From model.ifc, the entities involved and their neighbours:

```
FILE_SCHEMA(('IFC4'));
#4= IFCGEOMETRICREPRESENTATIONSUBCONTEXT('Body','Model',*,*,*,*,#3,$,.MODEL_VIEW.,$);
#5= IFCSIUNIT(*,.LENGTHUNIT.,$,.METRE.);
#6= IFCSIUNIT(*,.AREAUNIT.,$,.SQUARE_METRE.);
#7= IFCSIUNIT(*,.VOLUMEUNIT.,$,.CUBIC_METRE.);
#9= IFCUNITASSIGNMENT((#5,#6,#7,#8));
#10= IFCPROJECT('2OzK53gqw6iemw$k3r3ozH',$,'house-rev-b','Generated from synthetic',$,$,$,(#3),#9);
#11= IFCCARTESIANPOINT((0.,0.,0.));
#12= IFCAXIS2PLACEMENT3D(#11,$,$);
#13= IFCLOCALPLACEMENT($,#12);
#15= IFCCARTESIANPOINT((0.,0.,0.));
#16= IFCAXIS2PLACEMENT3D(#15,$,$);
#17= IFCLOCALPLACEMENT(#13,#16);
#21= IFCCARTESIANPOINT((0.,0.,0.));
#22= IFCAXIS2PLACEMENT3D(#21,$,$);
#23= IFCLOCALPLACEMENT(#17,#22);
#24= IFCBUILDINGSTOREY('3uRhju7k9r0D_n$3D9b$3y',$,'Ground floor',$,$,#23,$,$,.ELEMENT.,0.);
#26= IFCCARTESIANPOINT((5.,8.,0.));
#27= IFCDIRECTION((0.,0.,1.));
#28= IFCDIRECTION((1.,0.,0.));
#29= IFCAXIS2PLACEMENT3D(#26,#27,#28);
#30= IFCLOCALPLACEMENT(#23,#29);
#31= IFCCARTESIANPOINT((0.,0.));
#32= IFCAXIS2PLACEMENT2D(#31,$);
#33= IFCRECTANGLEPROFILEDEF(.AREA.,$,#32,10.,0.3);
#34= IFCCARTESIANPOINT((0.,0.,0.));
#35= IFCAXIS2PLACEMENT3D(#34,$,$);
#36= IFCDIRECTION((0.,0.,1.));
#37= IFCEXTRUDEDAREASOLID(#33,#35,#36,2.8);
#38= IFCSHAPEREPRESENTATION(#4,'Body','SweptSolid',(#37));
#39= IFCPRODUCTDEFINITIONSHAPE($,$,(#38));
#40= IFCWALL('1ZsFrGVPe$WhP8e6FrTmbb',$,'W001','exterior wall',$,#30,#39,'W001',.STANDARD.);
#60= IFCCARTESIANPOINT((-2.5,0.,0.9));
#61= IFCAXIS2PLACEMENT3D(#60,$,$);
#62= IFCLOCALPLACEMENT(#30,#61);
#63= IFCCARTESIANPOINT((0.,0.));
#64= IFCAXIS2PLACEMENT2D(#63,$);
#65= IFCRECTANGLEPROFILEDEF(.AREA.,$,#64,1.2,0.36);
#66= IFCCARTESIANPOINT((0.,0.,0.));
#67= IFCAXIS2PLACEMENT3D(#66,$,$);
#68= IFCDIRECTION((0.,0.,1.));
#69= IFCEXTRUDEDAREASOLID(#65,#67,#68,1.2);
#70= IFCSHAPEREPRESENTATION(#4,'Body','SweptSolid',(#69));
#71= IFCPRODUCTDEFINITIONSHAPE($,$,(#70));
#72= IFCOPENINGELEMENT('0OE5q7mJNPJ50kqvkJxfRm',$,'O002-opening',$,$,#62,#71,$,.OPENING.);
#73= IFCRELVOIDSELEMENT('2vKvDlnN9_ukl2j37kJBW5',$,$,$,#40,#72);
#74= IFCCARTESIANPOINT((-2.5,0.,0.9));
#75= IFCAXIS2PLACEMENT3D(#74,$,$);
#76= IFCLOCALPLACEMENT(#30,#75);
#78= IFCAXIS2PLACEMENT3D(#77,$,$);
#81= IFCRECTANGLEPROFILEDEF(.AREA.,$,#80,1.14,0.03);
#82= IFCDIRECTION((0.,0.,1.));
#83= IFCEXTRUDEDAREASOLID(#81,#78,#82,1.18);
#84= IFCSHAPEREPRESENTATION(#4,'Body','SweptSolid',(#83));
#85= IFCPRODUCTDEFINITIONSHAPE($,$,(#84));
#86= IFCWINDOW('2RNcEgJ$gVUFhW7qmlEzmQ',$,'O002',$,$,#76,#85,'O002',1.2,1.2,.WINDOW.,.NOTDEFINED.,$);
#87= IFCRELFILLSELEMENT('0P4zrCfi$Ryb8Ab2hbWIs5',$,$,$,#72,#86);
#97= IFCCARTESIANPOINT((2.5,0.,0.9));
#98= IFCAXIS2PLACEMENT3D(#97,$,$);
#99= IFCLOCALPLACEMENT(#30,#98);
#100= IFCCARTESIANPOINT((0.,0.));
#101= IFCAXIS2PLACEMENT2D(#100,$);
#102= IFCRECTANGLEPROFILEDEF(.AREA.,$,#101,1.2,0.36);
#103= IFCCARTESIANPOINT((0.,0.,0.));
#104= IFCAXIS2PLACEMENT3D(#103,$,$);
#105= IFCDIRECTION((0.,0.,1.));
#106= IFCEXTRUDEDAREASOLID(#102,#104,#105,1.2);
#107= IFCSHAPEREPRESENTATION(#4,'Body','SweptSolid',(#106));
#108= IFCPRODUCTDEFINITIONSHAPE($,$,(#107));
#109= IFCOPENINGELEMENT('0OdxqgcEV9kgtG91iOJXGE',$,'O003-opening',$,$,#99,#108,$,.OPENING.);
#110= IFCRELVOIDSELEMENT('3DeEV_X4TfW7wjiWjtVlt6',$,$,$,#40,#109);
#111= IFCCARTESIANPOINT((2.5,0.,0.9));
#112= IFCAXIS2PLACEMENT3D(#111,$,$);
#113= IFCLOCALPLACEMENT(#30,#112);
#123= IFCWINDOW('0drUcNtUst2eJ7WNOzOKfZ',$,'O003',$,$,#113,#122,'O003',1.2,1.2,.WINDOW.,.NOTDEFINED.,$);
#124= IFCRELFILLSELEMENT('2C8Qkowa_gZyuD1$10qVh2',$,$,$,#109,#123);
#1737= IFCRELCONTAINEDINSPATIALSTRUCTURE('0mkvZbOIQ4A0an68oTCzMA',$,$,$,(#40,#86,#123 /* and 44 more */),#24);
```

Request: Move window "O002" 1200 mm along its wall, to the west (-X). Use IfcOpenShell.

```python
import ifcopenshell
import ifcopenshell.api.geometry
import ifcopenshell.util.placement
import ifcopenshell.util.unit

model = ifcopenshell.open("model.ifc")
unit_scale = ifcopenshell.util.unit.calculate_unit_scale(model)

window = model.by_guid("2RNcEgJ$gVUFhW7qmlEzmQ")
opening = window.FillsVoids[0].RelatingOpeningElement
wall = opening.VoidsElements[0].RelatingBuildingElement

wall_matrix = ifcopenshell.util.placement.get_local_placement(wall.ObjectPlacement)
shift = wall_matrix[:3, 0] * -1.2 / unit_scale
before = ifcopenshell.util.placement.get_local_placement(window.ObjectPlacement)[:3, 3].copy()

# The window is not placed relative to its opening, so move both.
for product in (opening, window):
    matrix = ifcopenshell.util.placement.get_local_placement(product.ObjectPlacement)
    matrix[:3, 3] += shift
    ifcopenshell.api.geometry.edit_object_placement(model, product=product, matrix=matrix, is_si=False)

after = ifcopenshell.util.placement.get_local_placement(window.ObjectPlacement)[:3, 3]
print("window moved by", (after - before).round(3) + 0.0)

model.write("model_v2.ifc")
```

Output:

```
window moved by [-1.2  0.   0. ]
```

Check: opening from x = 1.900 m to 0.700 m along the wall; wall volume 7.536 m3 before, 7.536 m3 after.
